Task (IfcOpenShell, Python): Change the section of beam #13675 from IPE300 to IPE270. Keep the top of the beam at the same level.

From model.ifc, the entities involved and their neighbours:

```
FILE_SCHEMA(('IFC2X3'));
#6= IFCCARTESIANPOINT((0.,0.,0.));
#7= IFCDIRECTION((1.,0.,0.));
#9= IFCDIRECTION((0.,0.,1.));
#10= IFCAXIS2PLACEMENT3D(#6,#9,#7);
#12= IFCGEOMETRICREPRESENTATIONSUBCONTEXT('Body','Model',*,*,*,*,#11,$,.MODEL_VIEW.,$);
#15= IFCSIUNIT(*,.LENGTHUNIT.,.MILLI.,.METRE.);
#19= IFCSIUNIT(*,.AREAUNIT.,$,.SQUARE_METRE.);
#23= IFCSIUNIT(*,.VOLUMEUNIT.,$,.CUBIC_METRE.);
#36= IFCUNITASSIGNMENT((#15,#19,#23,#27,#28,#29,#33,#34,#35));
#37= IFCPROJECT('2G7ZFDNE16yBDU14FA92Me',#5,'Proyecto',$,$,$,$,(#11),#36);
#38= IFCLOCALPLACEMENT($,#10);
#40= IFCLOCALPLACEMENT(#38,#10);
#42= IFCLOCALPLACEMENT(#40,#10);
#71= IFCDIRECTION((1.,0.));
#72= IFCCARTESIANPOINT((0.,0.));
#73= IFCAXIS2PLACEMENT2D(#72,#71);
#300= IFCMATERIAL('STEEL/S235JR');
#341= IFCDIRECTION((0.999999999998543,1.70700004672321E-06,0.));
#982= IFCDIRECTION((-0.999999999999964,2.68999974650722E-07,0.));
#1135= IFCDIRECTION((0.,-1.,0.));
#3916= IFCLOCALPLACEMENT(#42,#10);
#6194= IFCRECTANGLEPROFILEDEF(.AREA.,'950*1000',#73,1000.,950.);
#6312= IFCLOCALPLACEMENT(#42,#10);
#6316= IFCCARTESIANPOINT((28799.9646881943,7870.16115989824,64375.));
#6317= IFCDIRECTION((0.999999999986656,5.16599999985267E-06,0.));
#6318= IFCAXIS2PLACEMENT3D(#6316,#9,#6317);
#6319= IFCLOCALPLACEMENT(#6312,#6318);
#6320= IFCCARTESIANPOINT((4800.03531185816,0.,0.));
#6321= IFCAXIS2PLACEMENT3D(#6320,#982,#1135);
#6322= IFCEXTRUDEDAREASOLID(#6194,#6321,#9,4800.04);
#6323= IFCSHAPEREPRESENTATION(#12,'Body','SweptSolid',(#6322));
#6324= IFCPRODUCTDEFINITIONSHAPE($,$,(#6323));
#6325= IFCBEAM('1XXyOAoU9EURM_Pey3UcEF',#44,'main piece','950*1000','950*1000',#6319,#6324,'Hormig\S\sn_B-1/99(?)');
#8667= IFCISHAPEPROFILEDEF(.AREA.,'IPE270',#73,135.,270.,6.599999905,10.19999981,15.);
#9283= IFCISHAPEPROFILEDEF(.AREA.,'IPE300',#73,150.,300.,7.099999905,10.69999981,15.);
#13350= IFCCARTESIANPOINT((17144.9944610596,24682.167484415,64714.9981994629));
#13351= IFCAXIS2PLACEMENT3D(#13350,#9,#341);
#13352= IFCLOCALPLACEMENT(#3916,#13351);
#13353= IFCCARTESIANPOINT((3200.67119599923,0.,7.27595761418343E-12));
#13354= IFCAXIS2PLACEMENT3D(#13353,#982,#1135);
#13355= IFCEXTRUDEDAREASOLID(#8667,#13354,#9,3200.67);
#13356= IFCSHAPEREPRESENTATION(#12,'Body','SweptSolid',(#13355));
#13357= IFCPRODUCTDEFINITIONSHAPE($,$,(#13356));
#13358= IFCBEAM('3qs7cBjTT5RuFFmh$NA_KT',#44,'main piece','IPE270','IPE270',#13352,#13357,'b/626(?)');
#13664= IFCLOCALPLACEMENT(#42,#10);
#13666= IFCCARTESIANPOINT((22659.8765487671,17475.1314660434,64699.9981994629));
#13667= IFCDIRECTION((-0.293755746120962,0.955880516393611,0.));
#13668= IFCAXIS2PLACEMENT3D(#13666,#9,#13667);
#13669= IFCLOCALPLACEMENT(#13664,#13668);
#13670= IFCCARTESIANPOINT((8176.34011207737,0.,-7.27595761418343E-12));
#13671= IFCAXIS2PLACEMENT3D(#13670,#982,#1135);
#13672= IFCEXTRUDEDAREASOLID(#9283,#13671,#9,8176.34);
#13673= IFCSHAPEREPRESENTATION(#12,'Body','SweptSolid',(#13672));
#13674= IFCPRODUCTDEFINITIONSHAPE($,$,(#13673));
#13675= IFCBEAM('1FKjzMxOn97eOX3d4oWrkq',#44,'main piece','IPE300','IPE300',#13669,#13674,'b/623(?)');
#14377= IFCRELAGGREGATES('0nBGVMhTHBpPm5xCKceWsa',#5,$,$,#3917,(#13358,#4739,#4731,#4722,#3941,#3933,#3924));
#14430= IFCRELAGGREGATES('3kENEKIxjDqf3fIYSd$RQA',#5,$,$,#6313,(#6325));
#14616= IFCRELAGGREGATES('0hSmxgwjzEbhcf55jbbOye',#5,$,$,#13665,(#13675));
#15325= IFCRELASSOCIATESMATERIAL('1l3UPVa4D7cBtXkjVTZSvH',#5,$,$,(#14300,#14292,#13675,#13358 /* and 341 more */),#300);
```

```python
import ifcopenshell
import ifcopenshell.util.element
import ifcopenshell.util.representation

model = ifcopenshell.open("model.ifc")

member = model.by_guid("1FKjzMxOn97eOX3d4oWrkq")
source = next(p for p in model.by_type("IfcIShapeProfileDef") if p.ProfileName == "IPE270")

body = ifcopenshell.util.representation.get_representation(member, "Model", "Body")
solid = body.Items[0]
old_profile = solid.SweptArea

# Copy the section's sizes but keep this member's own profile position.
profile = ifcopenshell.util.element.copy(model, source)
# Profiles are centred, so shift by half the change in depth to hold the top.
shift = (old_profile.OverallDepth - profile.OverallDepth) / 2
x, y = old_profile.Position.Location.Coordinates
up = (0.0, 1.0)  # upwards, in the solid's own plane
location = model.createIfcCartesianPoint((x + up[0] * shift, y + up[1] * shift))
profile.Position = model.createIfcAxis2Placement2D(location, old_profile.Position.RefDirection)
solid.SweptArea = profile
if not model.get_total_inverses(old_profile):
    ifcopenshell.util.element.remove_deep2(model, old_profile)
member.Description = member.Description.replace("IPE300", "IPE270")
member.ObjectType = member.ObjectType.replace("IPE300", "IPE270")

print(solid.SweptArea)

model.write("model-out.ifc")
```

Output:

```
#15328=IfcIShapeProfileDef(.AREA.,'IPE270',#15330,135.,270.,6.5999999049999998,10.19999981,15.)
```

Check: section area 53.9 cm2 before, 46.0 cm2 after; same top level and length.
